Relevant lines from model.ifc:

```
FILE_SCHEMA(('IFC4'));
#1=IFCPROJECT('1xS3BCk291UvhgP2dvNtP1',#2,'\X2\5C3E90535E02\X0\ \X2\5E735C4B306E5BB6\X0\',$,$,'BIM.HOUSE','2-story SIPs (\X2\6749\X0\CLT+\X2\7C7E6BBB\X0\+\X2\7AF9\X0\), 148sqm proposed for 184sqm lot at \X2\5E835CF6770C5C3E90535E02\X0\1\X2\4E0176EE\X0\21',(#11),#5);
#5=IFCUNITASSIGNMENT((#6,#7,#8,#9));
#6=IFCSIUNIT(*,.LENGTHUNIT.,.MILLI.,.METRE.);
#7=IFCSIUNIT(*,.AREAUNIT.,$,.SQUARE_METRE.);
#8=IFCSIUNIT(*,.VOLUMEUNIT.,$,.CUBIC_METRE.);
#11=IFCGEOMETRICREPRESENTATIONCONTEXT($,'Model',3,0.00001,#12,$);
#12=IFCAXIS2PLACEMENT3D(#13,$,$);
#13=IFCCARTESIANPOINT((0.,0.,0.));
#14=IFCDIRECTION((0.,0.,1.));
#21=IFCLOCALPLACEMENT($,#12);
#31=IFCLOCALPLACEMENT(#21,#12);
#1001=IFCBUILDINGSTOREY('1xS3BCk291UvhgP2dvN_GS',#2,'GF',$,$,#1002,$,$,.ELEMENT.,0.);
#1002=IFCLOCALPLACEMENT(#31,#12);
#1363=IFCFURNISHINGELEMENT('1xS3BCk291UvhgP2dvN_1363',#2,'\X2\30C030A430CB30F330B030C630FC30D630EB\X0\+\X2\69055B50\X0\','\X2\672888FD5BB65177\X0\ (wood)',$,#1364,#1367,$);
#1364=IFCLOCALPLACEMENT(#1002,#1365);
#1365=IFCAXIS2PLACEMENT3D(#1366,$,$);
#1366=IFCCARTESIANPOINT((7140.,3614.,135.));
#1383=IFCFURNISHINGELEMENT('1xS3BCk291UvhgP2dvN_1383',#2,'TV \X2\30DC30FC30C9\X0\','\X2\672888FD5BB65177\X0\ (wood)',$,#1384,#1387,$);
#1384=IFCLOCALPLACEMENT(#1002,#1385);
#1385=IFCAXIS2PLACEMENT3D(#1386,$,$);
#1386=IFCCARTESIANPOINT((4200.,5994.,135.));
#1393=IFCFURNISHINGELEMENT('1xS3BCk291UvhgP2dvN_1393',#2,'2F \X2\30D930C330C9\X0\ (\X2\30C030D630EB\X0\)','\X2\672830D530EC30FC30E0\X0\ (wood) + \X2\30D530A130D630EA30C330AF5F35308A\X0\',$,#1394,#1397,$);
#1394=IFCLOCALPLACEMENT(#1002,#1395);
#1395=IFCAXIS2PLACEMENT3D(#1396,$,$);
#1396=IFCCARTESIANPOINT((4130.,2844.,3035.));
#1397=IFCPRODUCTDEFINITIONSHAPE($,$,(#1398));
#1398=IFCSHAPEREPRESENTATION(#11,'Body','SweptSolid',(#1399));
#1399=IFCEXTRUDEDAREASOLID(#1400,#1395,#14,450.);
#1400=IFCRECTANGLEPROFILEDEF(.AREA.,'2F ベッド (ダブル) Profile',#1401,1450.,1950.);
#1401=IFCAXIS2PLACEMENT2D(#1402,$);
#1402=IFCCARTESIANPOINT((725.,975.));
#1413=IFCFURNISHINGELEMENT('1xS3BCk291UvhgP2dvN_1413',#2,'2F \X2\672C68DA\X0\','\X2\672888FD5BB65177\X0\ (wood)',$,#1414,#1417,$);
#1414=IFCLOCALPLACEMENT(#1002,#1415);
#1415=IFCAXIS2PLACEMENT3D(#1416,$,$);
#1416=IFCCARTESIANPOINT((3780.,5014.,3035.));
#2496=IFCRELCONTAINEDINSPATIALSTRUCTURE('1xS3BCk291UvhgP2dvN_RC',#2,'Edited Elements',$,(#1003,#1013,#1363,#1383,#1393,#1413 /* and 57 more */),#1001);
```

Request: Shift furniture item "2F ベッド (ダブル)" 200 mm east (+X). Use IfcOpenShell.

```python
import ifcopenshell
import ifcopenshell.api.geometry
import ifcopenshell.util.placement

model = ifcopenshell.open("model.ifc")

item = model.by_guid("1xS3BCk291UvhgP2dvN_1393")
matrix = ifcopenshell.util.placement.get_local_placement(item.ObjectPlacement)
matrix[0, 3] += 200.0
ifcopenshell.api.geometry.edit_object_placement(model, product=item, matrix=matrix, is_si=False)

print(ifcopenshell.util.placement.get_local_placement(item.ObjectPlacement).round(3) + 0.0)

model.write("model_edited.ifc")
```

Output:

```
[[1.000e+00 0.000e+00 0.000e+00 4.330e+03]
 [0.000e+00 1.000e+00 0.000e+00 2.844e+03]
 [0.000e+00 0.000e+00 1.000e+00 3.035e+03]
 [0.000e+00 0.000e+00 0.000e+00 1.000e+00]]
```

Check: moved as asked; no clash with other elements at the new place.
